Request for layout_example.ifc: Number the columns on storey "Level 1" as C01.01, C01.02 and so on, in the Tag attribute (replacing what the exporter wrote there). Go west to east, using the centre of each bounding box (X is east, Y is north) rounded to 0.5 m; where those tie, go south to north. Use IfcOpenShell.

First a look at what the model holds.

```python
import ifcopenshell
import ifcopenshell.util.element
import ifcopenshell.util.placement

model = ifcopenshell.open("layout_example.ifc")
print(model.schema)
storey = next(s for s in model.by_type("IfcBuildingStorey") if s.Name == "Level 1")
columns = [e for e in ifcopenshell.util.element.get_decomposition(storey) if e.is_a("IfcColumn")]
for e in sorted(columns, key=lambda e: e.id()):
    origin = ifcopenshell.util.placement.get_local_placement(e.ObjectPlacement)[:3, 3]
    print(e.id(), e.Tag, e.Name, origin.round(2) + 0.0, sep=" | ")
```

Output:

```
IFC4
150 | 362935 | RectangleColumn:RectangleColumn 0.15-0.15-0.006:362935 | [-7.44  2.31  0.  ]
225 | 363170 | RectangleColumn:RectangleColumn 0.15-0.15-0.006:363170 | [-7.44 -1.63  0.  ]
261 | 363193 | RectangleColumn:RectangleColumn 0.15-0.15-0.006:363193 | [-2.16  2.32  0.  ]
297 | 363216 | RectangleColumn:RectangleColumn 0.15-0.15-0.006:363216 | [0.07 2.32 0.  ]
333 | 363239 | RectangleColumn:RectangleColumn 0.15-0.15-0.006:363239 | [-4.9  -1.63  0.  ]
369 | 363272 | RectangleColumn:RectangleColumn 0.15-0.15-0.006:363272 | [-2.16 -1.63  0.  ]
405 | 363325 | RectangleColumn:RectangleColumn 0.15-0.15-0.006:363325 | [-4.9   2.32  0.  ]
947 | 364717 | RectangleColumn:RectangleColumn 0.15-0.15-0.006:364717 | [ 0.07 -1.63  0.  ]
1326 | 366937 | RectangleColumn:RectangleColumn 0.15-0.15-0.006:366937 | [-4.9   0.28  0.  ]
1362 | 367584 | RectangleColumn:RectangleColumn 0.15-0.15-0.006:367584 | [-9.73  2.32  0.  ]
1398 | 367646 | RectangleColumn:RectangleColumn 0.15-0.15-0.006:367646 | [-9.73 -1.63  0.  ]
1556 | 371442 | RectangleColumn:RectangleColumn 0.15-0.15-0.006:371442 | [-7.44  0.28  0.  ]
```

```python
import ifcopenshell
import ifcopenshell.geom
import ifcopenshell.util.element
import ifcopenshell.util.shape

model = ifcopenshell.open("layout_example.ifc")
settings = ifcopenshell.geom.settings()
settings.set("use-world-coords", True)


def centre(element):
    shape = ifcopenshell.geom.create_shape(settings, element)
    return ifcopenshell.util.shape.get_bbox_centroid(shape.geometry)


storey = next(s for s in model.by_type("IfcBuildingStorey") if s.Name == "Level 1")
columns = [e for e in ifcopenshell.util.element.get_decomposition(storey) if e.is_a("IfcColumn")]

# Insertion points can sit at a corner or the storey origin, so sort by the geometry (in metres).
centres = {e: centre(e) for e in columns}
columns.sort(key=lambda e: (round(centres[e][0] / 0.5), centres[e][1]))

for i, e in enumerate(columns, start=1):
    number = f"C01.{i:02d}"
    e.Tag = number
    print(e.id(), number)

model.write("layout_example_edited.ifc")
```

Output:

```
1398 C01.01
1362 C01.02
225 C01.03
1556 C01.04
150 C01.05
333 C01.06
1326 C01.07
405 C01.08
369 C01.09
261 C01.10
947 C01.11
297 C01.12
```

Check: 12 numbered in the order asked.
